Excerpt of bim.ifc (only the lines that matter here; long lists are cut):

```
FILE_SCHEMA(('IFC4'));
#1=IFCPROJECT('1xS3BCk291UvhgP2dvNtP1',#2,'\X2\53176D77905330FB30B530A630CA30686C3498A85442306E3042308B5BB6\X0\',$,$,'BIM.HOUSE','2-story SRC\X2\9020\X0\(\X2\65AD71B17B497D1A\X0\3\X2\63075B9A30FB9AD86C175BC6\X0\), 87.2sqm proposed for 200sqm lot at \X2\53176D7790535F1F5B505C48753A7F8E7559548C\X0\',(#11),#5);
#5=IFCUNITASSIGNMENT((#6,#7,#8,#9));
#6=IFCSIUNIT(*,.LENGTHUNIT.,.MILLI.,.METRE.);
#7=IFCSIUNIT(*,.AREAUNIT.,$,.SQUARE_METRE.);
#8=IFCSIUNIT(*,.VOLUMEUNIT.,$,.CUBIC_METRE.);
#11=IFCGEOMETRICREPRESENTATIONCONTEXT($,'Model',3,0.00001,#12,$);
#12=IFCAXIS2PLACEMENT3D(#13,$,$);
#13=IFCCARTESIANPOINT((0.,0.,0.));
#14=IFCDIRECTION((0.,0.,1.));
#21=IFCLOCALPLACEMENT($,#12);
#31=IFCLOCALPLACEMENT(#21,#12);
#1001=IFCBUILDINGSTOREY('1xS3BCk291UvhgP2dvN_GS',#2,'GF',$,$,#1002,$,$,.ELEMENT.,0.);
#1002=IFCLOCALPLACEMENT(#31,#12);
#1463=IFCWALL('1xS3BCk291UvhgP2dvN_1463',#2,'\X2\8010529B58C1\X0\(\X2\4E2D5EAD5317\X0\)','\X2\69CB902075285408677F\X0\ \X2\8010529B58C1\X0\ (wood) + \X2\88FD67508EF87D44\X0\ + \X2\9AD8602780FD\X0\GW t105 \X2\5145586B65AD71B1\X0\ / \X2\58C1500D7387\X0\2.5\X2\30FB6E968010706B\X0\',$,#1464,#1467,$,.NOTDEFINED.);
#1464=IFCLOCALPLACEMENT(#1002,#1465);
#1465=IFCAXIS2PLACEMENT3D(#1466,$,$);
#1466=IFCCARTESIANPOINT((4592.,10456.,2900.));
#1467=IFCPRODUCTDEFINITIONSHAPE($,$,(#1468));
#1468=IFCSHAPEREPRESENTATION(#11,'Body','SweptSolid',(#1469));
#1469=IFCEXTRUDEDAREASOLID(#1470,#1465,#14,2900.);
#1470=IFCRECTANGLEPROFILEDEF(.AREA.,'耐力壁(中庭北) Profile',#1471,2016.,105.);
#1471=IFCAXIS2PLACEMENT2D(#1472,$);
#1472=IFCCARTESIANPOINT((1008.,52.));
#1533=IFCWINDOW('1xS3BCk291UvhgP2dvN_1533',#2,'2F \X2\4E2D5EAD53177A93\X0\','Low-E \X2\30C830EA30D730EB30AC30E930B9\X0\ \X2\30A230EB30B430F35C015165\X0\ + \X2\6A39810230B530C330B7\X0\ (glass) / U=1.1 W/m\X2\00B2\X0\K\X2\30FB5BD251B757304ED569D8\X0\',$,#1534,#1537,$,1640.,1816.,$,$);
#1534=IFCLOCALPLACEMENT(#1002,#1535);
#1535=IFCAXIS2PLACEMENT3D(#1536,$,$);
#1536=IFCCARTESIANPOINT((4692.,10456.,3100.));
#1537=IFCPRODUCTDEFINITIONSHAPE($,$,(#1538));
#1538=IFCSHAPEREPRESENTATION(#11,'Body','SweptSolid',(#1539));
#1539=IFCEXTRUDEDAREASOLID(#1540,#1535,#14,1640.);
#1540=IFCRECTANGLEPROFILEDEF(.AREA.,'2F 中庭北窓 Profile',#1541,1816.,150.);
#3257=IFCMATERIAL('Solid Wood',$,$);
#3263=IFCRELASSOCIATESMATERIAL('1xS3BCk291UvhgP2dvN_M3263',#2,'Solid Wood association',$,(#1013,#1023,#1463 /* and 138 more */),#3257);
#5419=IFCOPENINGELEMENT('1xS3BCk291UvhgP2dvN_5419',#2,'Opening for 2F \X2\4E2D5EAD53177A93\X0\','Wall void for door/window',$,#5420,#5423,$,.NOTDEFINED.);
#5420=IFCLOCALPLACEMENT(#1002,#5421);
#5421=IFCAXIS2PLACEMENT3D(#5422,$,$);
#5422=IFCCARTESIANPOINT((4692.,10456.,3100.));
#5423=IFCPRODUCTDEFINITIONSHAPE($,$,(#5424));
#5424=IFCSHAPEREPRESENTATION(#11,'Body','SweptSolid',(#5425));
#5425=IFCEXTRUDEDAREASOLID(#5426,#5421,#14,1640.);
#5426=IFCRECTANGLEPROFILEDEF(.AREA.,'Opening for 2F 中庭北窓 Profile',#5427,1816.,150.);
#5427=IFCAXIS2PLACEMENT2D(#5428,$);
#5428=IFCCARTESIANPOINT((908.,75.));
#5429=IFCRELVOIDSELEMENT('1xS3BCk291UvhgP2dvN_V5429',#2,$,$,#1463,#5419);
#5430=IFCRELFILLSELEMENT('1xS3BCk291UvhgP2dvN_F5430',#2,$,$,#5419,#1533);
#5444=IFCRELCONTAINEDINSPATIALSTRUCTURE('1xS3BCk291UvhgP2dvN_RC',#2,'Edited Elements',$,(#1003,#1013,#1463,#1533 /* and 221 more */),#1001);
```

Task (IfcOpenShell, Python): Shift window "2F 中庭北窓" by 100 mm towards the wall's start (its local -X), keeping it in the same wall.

```python
import ifcopenshell
import ifcopenshell.api.geometry
import ifcopenshell.util.placement
import ifcopenshell.util.unit

model = ifcopenshell.open("bim.ifc")
unit_scale = ifcopenshell.util.unit.calculate_unit_scale(model)

window = model.by_id(1533)
opening = window.FillsVoids[0].RelatingOpeningElement
wall = opening.VoidsElements[0].RelatingBuildingElement

wall_matrix = ifcopenshell.util.placement.get_local_placement(wall.ObjectPlacement)
shift = wall_matrix[:3, 0] * -0.1 / unit_scale
before = ifcopenshell.util.placement.get_local_placement(window.ObjectPlacement)[:3, 3].copy()

# The window is not placed relative to its opening, so move both.
for product in (opening, window):
    matrix = ifcopenshell.util.placement.get_local_placement(product.ObjectPlacement)
    matrix[:3, 3] += shift
    ifcopenshell.api.geometry.edit_object_placement(model, product=product, matrix=matrix, is_si=False)

after = ifcopenshell.util.placement.get_local_placement(window.ObjectPlacement)[:3, 3]
print("window moved by", (after - before).round(3) + 0.0)

model.write("bim_updated.ifc")
```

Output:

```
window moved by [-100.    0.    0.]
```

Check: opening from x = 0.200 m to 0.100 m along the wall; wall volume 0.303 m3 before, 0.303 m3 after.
